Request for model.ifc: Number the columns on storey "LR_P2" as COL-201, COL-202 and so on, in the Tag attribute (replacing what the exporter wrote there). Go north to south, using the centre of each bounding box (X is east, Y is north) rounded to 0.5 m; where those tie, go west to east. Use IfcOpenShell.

First a look at what the model holds.

```python
import ifcopenshell
import ifcopenshell.util.element
import ifcopenshell.util.placement

model = ifcopenshell.open("model.ifc")
print(model.schema)
storey = next(s for s in model.by_type("IfcBuildingStorey") if s.Name == "LR_P2")
columns = [e for e in ifcopenshell.util.element.get_decomposition(storey) if e.is_a("IfcColumn")]
for e in sorted(columns, key=lambda e: e.id()):
    origin = ifcopenshell.util.placement.get_local_placement(e.ObjectPlacement)[:3, 3]
    print(e.id(), e.Tag, e.Name, origin.round(2) + 0.0, sep=" | ")
```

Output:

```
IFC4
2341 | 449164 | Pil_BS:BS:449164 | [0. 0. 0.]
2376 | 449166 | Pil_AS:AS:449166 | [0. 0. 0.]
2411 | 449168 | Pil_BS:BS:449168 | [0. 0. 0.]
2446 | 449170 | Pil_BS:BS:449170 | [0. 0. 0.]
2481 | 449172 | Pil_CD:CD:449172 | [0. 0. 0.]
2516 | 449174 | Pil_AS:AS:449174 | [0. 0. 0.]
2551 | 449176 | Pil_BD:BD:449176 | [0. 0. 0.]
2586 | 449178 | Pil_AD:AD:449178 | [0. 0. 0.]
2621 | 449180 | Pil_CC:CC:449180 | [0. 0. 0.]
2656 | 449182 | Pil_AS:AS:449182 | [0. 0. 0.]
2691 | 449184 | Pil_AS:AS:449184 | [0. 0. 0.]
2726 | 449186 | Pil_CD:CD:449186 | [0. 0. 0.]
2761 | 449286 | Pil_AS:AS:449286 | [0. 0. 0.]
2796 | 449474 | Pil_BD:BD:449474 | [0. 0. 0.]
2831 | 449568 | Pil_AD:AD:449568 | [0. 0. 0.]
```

```python
import ifcopenshell
import ifcopenshell.geom
import ifcopenshell.util.element
import ifcopenshell.util.shape

model = ifcopenshell.open("model.ifc")
settings = ifcopenshell.geom.settings()
settings.set("use-world-coords", True)


def centre(element):
    shape = ifcopenshell.geom.create_shape(settings, element)
    return ifcopenshell.util.shape.get_bbox_centroid(shape.geometry)


storey = next(s for s in model.by_type("IfcBuildingStorey") if s.Name == "LR_P2")
columns = [e for e in ifcopenshell.util.element.get_decomposition(storey) if e.is_a("IfcColumn")]

# Insertion points can sit at a corner or the storey origin, so sort by the geometry (in metres).
centres = {e: centre(e) for e in columns}
columns.sort(key=lambda e: (-round(centres[e][1] / 0.5), centres[e][0]))

for i, e in enumerate(columns, start=1):
    number = f"COL-2{i:02d}"
    e.Tag = number
    print(e.id(), number)

model.write("model_rev.ifc")
```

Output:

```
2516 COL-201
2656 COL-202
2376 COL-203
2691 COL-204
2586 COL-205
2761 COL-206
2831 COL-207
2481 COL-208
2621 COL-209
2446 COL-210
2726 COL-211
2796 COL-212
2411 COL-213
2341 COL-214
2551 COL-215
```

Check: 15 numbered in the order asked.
